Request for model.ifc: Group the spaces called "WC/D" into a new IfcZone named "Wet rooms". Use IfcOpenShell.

First a look at what the model holds.

```python
import ifcopenshell

model = ifcopenshell.open("model.ifc")
print(model.schema)
seen = {}
for space in model.by_type("IfcSpace"):
    seen[space.LongName] = seen.get(space.LongName, 0) + 1
for name, count in sorted(seen.items(), key=str):
    print(count, "x", name)
print("zones:", [z.Name for z in model.by_type("IfcZone")][:20])
```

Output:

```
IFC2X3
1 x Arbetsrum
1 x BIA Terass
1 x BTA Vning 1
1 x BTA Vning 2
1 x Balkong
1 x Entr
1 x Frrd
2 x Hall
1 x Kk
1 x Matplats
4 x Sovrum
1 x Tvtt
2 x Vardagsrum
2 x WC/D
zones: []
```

```python
import ifcopenshell
import ifcopenshell.api.group
import ifcopenshell.api.root

model = ifcopenshell.open("model.ifc")

names = {"WC/D"}
spaces = [s for s in model.by_type("IfcSpace") if s.LongName in names]

zone = ifcopenshell.api.root.create_entity(model, ifc_class="IfcZone", name="Wet rooms")
ifcopenshell.api.group.assign_group(model, products=spaces, group=zone)
print(len(spaces), "spaces in", zone.Name)

model.write("model_updated.ifc")
```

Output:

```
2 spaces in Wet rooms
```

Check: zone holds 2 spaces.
